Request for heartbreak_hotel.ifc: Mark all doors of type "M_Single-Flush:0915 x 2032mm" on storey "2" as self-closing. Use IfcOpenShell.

First a look at what the model holds.

```python
import ifcopenshell
import ifcopenshell.util.element

model = ifcopenshell.open("heartbreak_hotel.ifc")
print(model.schema)
storey = next(s for s in model.by_type("IfcBuildingStorey") if s.Name == "2")
doors = [e for e in ifcopenshell.util.element.get_decomposition(storey) if e.is_a("IfcDoor")]
seen = {}
for e in doors:
    element_type = ifcopenshell.util.element.get_type(e)
    key = (element_type.Name if element_type != e and element_type else None, ifcopenshell.util.element.get_pset(e, "Pset_DoorCommon", "SelfClosing"))
    seen[key] = seen.get(key, 0) + 1
for (name, value), count in sorted(seen.items(), key=str):
    print(count, "x", name, "|", value)
```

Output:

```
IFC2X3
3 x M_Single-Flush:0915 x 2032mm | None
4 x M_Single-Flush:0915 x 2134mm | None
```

```python
import ifcopenshell
import ifcopenshell.api.pset
import ifcopenshell.util.element

model = ifcopenshell.open("heartbreak_hotel.ifc")

storey = next(s for s in model.by_type("IfcBuildingStorey") if s.Name == "2")
doors = [e for e in ifcopenshell.util.element.get_decomposition(storey) if e.is_a("IfcDoor")]

count = 0
for e in doors:
    element_type = ifcopenshell.util.element.get_type(e)
    if element_type in (None, e) or element_type.Name != "M_Single-Flush:0915 x 2032mm":
        continue
    # add_pset returns the element's existing set when there is one.
    pset = ifcopenshell.api.pset.add_pset(model, product=e, name="Pset_DoorCommon")
    ifcopenshell.api.pset.edit_pset(model, pset=pset, properties={"SelfClosing": True})
    count += 1

print(count, "doors updated")

model.write("heartbreak_hotel_rev.ifc")
```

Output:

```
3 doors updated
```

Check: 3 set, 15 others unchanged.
